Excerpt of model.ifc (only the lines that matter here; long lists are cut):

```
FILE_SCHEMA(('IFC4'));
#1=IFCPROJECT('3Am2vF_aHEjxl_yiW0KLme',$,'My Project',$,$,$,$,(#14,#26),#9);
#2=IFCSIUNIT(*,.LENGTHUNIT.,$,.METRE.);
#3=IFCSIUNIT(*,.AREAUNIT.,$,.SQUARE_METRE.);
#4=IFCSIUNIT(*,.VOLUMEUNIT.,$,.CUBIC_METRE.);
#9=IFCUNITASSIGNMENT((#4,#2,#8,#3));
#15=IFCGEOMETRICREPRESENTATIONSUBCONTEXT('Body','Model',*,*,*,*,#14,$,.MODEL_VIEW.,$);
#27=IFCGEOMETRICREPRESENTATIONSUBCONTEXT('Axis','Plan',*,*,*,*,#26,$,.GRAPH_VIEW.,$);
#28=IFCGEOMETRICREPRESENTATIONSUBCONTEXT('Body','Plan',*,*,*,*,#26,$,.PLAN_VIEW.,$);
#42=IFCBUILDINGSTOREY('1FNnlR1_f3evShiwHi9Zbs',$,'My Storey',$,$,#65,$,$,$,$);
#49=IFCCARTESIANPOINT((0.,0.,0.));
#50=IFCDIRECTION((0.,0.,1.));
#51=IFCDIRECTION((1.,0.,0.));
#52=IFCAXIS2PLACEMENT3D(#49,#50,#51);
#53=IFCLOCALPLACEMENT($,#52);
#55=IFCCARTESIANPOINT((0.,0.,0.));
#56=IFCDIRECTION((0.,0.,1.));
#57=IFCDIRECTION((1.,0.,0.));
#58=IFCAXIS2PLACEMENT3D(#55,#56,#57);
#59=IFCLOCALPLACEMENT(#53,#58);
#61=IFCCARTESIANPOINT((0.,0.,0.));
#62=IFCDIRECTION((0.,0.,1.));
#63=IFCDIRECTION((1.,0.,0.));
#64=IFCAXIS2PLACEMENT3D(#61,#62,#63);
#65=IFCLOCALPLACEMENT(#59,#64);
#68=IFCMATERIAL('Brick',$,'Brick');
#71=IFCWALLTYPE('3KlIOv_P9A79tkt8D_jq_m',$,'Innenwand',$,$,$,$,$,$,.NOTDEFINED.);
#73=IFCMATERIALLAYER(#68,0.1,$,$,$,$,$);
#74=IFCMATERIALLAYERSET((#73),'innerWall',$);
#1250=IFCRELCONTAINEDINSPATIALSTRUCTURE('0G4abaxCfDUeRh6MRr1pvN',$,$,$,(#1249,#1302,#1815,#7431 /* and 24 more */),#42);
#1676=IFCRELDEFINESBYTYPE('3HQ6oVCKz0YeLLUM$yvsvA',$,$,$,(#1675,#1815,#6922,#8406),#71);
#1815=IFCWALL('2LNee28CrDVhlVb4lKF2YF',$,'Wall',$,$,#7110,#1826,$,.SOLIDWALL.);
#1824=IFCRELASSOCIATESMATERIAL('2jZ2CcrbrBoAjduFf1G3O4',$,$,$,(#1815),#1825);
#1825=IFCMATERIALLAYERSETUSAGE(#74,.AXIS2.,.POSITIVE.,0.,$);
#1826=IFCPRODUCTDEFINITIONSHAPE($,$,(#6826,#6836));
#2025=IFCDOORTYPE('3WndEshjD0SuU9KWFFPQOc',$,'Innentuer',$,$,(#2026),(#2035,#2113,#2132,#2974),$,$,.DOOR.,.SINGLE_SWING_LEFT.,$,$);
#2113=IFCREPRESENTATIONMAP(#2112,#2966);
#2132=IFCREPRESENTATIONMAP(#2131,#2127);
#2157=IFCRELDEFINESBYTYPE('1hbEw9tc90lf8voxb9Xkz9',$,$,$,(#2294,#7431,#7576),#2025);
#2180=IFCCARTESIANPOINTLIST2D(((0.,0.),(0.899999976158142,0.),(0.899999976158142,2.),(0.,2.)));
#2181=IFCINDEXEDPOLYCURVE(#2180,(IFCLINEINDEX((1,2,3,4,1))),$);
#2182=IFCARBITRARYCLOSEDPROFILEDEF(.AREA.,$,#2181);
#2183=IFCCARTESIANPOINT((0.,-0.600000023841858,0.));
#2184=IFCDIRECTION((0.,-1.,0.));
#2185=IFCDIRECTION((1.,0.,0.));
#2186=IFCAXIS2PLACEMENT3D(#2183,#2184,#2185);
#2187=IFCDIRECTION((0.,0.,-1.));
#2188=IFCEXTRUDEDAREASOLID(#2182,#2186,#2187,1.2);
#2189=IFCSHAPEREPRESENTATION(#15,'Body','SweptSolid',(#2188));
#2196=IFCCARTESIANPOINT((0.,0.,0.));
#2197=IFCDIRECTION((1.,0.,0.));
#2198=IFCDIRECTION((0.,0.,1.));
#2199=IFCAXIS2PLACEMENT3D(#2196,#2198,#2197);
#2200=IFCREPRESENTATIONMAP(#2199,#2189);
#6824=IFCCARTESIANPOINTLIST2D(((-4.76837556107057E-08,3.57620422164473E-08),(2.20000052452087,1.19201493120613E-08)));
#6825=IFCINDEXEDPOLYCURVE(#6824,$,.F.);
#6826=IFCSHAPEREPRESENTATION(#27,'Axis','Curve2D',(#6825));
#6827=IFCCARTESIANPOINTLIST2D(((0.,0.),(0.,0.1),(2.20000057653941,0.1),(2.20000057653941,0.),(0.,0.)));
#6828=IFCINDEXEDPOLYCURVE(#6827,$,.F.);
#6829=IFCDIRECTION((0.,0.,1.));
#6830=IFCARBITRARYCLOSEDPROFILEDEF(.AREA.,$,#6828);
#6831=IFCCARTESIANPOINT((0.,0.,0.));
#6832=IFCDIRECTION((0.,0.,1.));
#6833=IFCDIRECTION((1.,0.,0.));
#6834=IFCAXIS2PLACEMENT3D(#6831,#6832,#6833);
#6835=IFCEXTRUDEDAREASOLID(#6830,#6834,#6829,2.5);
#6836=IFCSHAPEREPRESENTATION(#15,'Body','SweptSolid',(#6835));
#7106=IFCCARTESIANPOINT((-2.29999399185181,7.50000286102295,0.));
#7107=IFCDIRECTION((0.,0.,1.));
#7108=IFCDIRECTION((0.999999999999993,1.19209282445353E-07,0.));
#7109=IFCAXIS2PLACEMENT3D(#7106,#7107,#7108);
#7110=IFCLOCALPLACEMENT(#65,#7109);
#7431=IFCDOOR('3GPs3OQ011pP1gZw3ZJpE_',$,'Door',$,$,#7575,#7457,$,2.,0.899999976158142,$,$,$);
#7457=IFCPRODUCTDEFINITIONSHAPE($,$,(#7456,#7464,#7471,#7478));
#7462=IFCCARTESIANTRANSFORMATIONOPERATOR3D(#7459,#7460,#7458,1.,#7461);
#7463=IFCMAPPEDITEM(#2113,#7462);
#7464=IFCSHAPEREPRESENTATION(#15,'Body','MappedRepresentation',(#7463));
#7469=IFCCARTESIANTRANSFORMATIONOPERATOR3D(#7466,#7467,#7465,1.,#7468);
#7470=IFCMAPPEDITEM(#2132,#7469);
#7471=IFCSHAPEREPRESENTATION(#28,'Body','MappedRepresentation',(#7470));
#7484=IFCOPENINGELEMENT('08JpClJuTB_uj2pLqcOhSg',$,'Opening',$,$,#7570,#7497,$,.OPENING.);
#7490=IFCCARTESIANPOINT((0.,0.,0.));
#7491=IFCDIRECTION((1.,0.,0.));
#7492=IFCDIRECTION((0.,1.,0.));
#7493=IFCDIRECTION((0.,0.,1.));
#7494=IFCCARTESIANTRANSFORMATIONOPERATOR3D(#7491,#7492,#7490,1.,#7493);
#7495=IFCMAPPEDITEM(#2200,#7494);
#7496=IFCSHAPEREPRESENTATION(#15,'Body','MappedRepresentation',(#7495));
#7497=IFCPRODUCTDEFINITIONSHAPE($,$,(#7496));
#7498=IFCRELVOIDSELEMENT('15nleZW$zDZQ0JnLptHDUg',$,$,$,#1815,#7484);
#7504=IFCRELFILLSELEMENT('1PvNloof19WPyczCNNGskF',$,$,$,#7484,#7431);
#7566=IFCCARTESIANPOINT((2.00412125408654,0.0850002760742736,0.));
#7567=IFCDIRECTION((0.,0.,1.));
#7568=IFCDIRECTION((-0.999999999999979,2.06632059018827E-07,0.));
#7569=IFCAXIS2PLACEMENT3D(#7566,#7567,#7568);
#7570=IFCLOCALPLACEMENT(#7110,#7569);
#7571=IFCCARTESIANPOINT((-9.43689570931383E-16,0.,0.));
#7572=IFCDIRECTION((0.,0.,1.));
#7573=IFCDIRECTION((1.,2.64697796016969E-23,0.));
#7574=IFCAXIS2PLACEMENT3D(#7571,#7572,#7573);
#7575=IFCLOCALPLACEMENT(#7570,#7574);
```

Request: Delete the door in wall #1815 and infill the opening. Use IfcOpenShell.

```python
import ifcopenshell
import ifcopenshell.api.feature
import ifcopenshell.api.root
import ifcopenshell.geom
import ifcopenshell.util.shape

model = ifcopenshell.open("model.ifc")
settings = ifcopenshell.geom.settings()


def volume(element):
    """Net volume in cubic metres, openings subtracted."""
    shape = ifcopenshell.geom.create_shape(settings, element)
    return ifcopenshell.util.shape.get_volume(shape.geometry)


door = model.by_id(7431)
opening = door.FillsVoids[0].RelatingOpeningElement
wall = opening.VoidsElements[0].RelatingBuildingElement
before = volume(wall)

ifcopenshell.api.root.remove_product(model, product=door)
ifcopenshell.api.feature.remove_feature(model, feature=opening)

after = volume(wall)

print(f"wall volume {before:.3f} -> {after:.3f} m3")

model.write("model_rev.ifc")
```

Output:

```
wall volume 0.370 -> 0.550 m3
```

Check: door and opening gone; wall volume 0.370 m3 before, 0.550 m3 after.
